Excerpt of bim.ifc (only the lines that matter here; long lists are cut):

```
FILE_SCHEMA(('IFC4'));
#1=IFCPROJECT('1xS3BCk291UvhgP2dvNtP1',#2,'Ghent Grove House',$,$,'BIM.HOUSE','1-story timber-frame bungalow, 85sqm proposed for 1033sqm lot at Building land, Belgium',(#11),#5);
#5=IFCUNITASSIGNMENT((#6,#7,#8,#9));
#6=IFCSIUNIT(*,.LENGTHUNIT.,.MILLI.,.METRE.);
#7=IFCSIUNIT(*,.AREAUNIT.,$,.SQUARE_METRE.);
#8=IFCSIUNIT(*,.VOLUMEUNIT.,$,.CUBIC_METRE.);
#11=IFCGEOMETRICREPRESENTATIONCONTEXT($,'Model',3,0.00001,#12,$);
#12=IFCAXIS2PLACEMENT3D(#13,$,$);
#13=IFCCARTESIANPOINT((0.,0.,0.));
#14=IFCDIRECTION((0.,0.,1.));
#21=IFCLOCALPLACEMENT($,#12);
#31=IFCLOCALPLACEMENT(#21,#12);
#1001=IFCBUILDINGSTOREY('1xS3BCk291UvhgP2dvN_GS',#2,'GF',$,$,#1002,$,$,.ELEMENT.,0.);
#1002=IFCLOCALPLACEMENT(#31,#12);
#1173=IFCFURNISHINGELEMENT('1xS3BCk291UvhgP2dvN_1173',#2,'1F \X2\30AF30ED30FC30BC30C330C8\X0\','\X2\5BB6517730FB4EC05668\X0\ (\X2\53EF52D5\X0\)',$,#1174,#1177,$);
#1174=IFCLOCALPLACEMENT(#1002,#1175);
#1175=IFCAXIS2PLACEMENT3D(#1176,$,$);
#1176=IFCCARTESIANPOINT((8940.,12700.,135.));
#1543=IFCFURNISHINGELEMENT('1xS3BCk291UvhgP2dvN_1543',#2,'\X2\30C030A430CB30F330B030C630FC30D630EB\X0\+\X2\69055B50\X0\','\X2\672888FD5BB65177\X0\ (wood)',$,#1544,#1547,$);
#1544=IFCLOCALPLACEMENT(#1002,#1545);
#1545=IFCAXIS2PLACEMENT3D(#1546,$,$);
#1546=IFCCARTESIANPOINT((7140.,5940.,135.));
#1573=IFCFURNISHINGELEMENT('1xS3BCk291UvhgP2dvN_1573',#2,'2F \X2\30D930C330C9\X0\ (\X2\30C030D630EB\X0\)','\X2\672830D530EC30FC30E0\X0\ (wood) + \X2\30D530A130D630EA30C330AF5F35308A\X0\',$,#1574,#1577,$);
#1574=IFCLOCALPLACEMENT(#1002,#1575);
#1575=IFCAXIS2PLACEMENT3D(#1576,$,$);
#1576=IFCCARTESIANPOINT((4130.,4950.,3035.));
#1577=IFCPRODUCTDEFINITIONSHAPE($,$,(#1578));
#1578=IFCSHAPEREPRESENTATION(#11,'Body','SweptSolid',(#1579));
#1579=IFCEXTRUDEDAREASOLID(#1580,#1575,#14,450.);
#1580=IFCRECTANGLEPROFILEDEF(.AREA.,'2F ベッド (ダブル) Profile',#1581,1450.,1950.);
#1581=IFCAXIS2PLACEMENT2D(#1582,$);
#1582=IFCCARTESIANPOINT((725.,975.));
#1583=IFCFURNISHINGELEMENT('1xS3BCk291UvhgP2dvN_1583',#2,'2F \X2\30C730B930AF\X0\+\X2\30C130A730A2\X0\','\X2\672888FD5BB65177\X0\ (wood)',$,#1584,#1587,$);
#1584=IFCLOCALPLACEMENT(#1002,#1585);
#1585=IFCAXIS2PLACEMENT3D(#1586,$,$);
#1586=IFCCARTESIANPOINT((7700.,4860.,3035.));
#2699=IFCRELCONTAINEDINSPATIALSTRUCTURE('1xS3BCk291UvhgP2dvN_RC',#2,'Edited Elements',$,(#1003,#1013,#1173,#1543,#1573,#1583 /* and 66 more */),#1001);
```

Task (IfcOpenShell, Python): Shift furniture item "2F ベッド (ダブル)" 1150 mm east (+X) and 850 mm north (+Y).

```python
import ifcopenshell
import ifcopenshell.api.geometry
import ifcopenshell.util.placement
import ifcopenshell.util.unit

model = ifcopenshell.open("bim.ifc")
unit_scale = ifcopenshell.util.unit.calculate_unit_scale(model)

item = model.by_id(1573)
matrix = ifcopenshell.util.placement.get_local_placement(item.ObjectPlacement)
matrix[0, 3] += 1.15 / unit_scale
matrix[1, 3] += 0.85 / unit_scale
ifcopenshell.api.geometry.edit_object_placement(model, product=item, matrix=matrix, is_si=False)

print(ifcopenshell.util.placement.get_local_placement(item.ObjectPlacement).round(3) + 0.0)

model.write("bim_edited.ifc")
```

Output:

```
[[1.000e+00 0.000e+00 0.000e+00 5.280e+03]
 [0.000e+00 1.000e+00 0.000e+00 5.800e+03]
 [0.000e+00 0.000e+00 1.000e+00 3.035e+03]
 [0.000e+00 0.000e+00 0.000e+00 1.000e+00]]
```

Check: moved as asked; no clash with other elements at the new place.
